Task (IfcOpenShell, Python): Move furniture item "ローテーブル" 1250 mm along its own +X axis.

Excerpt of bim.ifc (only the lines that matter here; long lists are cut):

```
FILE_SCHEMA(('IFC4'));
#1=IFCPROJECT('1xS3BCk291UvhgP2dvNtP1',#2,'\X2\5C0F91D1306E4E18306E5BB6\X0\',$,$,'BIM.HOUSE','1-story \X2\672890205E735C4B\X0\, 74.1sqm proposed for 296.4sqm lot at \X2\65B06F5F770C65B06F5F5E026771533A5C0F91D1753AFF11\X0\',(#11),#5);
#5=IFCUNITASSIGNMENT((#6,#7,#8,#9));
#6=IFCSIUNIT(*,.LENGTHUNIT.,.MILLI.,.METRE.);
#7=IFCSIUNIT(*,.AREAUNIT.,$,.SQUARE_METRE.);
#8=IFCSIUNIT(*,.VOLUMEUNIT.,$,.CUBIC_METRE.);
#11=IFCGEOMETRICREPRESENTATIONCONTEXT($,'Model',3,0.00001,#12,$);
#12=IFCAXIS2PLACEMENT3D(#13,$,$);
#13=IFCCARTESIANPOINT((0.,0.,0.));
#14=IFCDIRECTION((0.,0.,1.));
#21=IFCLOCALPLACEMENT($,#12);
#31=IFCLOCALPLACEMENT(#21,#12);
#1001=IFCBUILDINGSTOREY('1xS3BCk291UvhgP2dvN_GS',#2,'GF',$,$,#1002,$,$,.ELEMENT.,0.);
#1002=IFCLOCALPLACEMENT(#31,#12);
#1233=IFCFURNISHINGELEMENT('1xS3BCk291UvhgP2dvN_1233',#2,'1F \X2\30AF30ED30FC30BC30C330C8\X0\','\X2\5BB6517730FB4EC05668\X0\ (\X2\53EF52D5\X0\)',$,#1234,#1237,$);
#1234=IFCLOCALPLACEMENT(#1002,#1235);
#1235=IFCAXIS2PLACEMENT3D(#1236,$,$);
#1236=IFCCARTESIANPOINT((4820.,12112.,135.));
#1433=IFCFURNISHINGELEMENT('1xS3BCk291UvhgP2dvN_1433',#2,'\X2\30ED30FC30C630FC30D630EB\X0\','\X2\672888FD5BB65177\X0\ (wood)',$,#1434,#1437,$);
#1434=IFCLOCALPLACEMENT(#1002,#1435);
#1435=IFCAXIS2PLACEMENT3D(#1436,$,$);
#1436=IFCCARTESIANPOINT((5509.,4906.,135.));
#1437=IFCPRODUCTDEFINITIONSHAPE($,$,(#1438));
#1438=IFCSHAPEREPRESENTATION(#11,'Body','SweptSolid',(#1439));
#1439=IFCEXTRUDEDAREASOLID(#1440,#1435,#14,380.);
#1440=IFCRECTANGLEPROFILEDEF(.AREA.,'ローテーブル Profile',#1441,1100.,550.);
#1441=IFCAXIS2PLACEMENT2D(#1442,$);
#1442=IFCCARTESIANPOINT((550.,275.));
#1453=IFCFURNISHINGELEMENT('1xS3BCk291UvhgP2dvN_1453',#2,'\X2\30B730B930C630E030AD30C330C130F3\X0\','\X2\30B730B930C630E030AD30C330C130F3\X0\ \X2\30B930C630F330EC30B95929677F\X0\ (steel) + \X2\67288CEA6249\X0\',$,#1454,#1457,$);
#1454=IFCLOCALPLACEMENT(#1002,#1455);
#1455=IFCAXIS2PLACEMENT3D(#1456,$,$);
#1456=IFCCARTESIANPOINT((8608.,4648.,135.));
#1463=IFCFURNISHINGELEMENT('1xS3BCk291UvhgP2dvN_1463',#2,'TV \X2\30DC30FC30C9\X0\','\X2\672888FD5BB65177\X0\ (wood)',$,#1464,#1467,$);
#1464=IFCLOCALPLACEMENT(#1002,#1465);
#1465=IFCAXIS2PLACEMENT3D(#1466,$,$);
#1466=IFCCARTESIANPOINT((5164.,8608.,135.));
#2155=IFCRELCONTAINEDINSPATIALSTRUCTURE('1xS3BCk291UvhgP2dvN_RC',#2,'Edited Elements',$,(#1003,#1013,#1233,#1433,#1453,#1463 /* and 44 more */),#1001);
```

```python
import ifcopenshell
import ifcopenshell.api.geometry
import ifcopenshell.util.placement
import ifcopenshell.util.unit

model = ifcopenshell.open("bim.ifc")
unit_scale = ifcopenshell.util.unit.calculate_unit_scale(model)

item = model.by_id(1433)
matrix = ifcopenshell.util.placement.get_local_placement(item.ObjectPlacement)
matrix[:3, 3] += matrix[:3, 0] * 1.25 / unit_scale
ifcopenshell.api.geometry.edit_object_placement(model, product=item, matrix=matrix, is_si=False)

print(ifcopenshell.util.placement.get_local_placement(item.ObjectPlacement).round(3) + 0.0)

model.write("bim_updated.ifc")
```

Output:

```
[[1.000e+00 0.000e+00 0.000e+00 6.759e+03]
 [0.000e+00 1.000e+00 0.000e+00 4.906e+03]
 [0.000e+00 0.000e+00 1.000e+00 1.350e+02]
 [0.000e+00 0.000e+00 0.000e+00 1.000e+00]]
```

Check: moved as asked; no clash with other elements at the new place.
